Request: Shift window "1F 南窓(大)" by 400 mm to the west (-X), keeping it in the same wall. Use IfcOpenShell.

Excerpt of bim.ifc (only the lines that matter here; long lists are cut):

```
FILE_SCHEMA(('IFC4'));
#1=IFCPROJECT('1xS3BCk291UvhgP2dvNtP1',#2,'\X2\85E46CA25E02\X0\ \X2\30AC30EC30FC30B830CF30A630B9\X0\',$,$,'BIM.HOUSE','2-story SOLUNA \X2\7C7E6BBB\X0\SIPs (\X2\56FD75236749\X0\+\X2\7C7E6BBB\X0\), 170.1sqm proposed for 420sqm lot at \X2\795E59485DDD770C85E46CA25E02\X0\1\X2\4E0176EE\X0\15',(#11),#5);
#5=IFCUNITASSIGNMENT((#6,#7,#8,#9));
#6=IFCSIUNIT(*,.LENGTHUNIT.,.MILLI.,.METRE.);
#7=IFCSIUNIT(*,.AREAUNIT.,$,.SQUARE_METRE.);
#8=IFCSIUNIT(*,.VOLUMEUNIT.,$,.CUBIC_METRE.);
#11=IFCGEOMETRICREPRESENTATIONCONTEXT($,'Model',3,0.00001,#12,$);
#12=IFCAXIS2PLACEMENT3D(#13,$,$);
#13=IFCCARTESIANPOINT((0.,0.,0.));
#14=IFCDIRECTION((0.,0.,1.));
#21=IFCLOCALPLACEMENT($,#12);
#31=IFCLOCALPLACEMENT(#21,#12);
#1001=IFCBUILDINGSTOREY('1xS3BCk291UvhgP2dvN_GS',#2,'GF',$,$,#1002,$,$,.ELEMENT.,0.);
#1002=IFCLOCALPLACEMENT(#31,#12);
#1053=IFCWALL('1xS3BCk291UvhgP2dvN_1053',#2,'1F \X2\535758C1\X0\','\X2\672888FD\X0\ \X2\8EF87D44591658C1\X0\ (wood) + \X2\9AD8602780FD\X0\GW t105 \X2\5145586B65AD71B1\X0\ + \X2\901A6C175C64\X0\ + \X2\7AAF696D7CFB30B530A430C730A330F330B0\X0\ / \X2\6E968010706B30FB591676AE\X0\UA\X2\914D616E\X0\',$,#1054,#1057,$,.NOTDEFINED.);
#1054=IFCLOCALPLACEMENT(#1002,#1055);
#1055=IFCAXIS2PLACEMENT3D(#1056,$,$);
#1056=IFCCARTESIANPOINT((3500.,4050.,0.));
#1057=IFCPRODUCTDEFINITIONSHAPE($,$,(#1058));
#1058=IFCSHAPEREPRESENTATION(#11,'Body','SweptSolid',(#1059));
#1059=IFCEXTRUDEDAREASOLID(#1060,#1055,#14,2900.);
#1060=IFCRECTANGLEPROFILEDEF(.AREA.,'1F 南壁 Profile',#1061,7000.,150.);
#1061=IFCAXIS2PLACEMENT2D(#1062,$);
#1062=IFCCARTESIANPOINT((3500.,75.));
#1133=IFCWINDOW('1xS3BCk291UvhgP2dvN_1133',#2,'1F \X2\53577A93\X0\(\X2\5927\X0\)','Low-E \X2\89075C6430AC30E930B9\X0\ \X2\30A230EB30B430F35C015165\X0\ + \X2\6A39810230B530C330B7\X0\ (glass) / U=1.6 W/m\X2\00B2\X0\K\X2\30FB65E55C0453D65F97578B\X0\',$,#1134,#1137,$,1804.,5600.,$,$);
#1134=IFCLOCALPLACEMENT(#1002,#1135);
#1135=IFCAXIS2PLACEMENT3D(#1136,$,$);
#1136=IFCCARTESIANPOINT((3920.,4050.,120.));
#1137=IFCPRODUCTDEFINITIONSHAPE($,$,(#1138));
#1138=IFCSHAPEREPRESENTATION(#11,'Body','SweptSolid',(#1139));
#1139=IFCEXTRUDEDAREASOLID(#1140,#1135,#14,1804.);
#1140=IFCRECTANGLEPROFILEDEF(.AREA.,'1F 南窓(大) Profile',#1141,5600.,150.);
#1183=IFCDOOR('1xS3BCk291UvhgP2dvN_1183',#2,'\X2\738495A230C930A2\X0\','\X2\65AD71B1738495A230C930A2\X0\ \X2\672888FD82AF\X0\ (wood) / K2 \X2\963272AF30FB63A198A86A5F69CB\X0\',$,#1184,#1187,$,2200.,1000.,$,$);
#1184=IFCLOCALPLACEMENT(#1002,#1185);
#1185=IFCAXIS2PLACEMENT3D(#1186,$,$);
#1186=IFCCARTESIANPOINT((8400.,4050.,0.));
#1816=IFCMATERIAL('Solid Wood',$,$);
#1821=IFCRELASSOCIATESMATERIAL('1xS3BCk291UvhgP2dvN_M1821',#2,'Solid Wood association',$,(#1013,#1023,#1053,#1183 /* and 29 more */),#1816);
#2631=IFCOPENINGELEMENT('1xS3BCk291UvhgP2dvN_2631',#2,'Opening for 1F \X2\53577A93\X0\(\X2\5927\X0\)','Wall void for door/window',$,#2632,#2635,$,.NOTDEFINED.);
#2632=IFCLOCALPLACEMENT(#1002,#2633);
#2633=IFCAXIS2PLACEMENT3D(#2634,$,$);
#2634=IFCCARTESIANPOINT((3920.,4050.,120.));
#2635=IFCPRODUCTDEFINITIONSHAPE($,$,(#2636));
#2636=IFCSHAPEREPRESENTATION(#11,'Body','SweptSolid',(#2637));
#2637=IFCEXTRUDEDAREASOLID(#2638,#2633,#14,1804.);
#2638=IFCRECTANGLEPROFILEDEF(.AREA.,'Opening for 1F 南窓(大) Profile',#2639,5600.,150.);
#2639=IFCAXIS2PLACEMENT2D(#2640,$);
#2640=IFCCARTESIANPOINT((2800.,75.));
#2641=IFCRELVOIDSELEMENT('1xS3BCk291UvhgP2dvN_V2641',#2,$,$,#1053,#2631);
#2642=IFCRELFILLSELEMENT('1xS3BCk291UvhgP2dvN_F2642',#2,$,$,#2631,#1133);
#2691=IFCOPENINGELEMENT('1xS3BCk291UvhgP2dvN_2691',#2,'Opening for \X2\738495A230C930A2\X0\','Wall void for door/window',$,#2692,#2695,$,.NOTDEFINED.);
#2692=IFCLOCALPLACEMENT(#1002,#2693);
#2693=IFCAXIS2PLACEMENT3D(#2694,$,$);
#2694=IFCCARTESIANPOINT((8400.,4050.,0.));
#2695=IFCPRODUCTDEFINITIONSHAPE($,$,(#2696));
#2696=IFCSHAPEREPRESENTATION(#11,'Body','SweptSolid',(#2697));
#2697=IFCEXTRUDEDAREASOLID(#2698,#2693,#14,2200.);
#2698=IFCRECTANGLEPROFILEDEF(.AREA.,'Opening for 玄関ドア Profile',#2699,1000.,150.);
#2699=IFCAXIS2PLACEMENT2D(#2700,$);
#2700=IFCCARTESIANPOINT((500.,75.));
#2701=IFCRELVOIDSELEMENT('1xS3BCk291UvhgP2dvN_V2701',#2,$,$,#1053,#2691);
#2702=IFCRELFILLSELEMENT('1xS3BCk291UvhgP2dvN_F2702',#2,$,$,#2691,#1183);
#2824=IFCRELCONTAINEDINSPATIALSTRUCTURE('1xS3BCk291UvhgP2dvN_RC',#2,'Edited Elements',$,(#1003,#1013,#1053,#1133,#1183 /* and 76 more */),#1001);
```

```python
import ifcopenshell
import ifcopenshell.api.geometry
import ifcopenshell.util.placement
import ifcopenshell.util.unit

model = ifcopenshell.open("bim.ifc")
unit_scale = ifcopenshell.util.unit.calculate_unit_scale(model)

window = model.by_guid("1xS3BCk291UvhgP2dvN_1133")
opening = window.FillsVoids[0].RelatingOpeningElement
wall = opening.VoidsElements[0].RelatingBuildingElement

wall_matrix = ifcopenshell.util.placement.get_local_placement(wall.ObjectPlacement)
shift = wall_matrix[:3, 0] * -0.4 / unit_scale
before = ifcopenshell.util.placement.get_local_placement(window.ObjectPlacement)[:3, 3].copy()

# The window is not placed relative to its opening, so move both.
for product in (opening, window):
    matrix = ifcopenshell.util.placement.get_local_placement(product.ObjectPlacement)
    matrix[:3, 3] += shift
    ifcopenshell.api.geometry.edit_object_placement(model, product=product, matrix=matrix, is_si=False)

after = ifcopenshell.util.placement.get_local_placement(window.ObjectPlacement)[:3, 3]
print("window moved by", (after - before).round(3) + 0.0)

model.write("bim_v2.ifc")
```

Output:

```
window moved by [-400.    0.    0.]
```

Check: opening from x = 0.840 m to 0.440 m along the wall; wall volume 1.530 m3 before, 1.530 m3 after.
